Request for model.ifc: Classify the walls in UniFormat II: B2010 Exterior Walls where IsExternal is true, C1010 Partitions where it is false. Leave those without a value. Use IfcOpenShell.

First a look at what the model holds.

```python
import ifcopenshell
import ifcopenshell.util.element

model = ifcopenshell.open("model.ifc")
print(model.schema)
print("classifications:", [c.Name for c in model.by_type("IfcClassification")])
values = [ifcopenshell.util.element.get_pset(e, "Pset_WallCommon", "IsExternal") for e in model.by_type("IfcWall")]
for value in (True, False, None):
    print("IsExternal", value, values.count(value))
```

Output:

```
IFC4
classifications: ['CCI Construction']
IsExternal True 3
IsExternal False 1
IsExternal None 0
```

```python
import ifcopenshell
import ifcopenshell.api.classification
import ifcopenshell.util.element

model = ifcopenshell.open("model.ifc")

system = ifcopenshell.api.classification.add_classification(model, classification="UniFormat II")

walls = model.by_type("IfcWall")
external = {e: ifcopenshell.util.element.get_pset(e, "Pset_WallCommon", "IsExternal") for e in walls}
for flag, code, name in ((True, "B2010", "Exterior Walls"), (False, "C1010", "Partitions")):
    products = [e for e in walls if external[e] is flag]
    ifcopenshell.api.classification.add_reference(
        model, products=products, classification=system, identification=code, name=name
    )
    print(code, len(products))

model.write("model-out.ifc")
```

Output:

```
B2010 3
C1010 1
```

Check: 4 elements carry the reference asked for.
